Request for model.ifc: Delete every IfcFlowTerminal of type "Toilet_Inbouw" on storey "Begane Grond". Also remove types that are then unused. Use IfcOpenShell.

First a look at what the model holds.

```python
import ifcopenshell
import ifcopenshell.util.element

model = ifcopenshell.open("model.ifc")
print(model.schema)
storey = next(s for s in model.by_type("IfcBuildingStorey") if s.Name == "Begane Grond")
terminals = [e for e in ifcopenshell.util.element.get_decomposition(storey) if e.is_a("IfcFlowTerminal")]
seen = {}
for e in terminals:
    element_type = ifcopenshell.util.element.get_type(e)
    name = element_type.Name if element_type not in (None, e) else None
    seen[name] = seen.get(name, 0) + 1
for name, count in sorted(seen.items(), key=str):
    print(count, "x", name)
```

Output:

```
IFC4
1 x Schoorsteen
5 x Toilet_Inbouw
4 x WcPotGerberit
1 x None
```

```python
import ifcopenshell
import ifcopenshell.api.root
import ifcopenshell.util.element

model = ifcopenshell.open("model.ifc")

storey = next(s for s in model.by_type("IfcBuildingStorey") if s.Name == "Begane Grond")
terminals = [e for e in ifcopenshell.util.element.get_decomposition(storey) if e.is_a("IfcFlowTerminal")]
targets = [e for e in terminals if (t := ifcopenshell.util.element.get_type(e)) not in (None, e) and t.Name == "Toilet_Inbouw"]
types = {ifcopenshell.util.element.get_type(e) for e in targets} - {None, *targets}

for e in targets:
    ifcopenshell.api.root.remove_product(model, product=e)
print(len(targets), "removed")

unused = [t for t in types if not ifcopenshell.util.element.get_types(t)]
for t in unused:
    ifcopenshell.api.root.remove_product(model, product=t)
print(len(unused), "unused types removed")

model.write("model_v2.ifc")
```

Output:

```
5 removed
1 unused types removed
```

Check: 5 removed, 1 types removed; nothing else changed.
